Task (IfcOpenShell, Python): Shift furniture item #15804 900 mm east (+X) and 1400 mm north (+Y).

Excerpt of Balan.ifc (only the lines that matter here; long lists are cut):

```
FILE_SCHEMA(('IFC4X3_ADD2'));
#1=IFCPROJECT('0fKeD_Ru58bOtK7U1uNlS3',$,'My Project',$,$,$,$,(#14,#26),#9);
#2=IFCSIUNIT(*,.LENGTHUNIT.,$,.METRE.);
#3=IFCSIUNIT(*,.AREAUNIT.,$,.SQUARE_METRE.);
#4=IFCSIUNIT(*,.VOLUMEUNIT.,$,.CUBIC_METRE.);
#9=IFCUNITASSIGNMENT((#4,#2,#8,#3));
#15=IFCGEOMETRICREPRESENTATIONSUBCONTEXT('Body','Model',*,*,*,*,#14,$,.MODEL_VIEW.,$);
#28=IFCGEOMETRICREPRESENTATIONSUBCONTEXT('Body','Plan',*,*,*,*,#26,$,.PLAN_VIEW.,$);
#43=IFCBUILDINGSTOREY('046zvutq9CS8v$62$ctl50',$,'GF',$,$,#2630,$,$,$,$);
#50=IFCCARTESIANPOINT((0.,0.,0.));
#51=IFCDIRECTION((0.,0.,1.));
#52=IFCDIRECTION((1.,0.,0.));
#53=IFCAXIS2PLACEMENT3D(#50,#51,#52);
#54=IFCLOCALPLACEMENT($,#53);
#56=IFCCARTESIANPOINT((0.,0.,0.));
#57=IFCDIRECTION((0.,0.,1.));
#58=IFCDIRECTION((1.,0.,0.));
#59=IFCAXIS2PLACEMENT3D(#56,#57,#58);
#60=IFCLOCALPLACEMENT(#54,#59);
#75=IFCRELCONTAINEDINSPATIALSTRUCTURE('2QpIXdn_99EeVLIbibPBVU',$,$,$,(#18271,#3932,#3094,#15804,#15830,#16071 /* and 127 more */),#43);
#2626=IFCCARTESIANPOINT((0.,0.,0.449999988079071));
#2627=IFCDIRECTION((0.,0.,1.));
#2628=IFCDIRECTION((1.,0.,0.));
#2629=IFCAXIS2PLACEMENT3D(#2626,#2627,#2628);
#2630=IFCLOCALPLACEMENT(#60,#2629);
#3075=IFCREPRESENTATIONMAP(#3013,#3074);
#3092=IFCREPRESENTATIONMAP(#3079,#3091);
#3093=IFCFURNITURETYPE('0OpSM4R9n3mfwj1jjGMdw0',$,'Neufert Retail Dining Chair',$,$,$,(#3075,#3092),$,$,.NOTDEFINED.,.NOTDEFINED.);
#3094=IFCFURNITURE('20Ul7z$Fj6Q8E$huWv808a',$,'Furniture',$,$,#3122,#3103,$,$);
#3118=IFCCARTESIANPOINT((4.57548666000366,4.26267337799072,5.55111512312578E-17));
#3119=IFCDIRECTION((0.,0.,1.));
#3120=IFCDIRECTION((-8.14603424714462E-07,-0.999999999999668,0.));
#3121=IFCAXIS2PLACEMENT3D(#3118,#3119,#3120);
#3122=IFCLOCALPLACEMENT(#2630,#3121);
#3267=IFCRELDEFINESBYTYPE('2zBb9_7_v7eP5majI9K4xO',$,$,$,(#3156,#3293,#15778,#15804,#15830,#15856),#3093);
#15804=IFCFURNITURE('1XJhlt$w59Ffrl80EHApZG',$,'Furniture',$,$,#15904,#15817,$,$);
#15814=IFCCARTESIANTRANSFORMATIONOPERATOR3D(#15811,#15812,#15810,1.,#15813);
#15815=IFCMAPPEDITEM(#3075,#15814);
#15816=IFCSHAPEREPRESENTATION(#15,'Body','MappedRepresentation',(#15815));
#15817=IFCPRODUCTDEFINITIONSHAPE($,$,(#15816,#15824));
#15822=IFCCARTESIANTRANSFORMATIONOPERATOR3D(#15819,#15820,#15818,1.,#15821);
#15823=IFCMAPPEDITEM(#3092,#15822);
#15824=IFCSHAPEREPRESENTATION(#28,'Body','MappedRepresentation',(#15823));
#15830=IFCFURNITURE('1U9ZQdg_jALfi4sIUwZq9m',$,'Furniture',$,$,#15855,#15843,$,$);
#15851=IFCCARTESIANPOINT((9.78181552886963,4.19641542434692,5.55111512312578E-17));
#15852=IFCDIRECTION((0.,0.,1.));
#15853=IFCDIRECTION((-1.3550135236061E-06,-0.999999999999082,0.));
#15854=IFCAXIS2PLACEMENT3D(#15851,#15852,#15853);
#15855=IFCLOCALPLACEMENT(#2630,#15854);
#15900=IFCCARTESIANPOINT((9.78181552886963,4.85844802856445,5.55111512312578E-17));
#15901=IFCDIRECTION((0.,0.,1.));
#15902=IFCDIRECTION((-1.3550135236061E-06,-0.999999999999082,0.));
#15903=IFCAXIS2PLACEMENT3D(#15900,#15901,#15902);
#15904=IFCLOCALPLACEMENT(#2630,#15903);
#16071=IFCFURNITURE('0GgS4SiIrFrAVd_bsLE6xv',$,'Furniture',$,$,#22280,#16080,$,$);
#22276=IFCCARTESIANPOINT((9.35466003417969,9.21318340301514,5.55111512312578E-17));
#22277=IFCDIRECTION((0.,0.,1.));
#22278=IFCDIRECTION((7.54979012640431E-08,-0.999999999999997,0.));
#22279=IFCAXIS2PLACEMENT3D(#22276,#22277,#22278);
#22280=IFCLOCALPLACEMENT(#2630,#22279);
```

```python
import ifcopenshell
import ifcopenshell.api.geometry
import ifcopenshell.util.placement
import ifcopenshell.util.unit

model = ifcopenshell.open("Balan.ifc")
unit_scale = ifcopenshell.util.unit.calculate_unit_scale(model)

item = model.by_guid("1XJhlt$w59Ffrl80EHApZG")
matrix = ifcopenshell.util.placement.get_local_placement(item.ObjectPlacement)
matrix[0, 3] += 0.9 / unit_scale
matrix[1, 3] += 1.4 / unit_scale
ifcopenshell.api.geometry.edit_object_placement(model, product=item, matrix=matrix, is_si=False)

print(ifcopenshell.util.placement.get_local_placement(item.ObjectPlacement).round(3) + 0.0)

model.write("Balan_v2.ifc")
```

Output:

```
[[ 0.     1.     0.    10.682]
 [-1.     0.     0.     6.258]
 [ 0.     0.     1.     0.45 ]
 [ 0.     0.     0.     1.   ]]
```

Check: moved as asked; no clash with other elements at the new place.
